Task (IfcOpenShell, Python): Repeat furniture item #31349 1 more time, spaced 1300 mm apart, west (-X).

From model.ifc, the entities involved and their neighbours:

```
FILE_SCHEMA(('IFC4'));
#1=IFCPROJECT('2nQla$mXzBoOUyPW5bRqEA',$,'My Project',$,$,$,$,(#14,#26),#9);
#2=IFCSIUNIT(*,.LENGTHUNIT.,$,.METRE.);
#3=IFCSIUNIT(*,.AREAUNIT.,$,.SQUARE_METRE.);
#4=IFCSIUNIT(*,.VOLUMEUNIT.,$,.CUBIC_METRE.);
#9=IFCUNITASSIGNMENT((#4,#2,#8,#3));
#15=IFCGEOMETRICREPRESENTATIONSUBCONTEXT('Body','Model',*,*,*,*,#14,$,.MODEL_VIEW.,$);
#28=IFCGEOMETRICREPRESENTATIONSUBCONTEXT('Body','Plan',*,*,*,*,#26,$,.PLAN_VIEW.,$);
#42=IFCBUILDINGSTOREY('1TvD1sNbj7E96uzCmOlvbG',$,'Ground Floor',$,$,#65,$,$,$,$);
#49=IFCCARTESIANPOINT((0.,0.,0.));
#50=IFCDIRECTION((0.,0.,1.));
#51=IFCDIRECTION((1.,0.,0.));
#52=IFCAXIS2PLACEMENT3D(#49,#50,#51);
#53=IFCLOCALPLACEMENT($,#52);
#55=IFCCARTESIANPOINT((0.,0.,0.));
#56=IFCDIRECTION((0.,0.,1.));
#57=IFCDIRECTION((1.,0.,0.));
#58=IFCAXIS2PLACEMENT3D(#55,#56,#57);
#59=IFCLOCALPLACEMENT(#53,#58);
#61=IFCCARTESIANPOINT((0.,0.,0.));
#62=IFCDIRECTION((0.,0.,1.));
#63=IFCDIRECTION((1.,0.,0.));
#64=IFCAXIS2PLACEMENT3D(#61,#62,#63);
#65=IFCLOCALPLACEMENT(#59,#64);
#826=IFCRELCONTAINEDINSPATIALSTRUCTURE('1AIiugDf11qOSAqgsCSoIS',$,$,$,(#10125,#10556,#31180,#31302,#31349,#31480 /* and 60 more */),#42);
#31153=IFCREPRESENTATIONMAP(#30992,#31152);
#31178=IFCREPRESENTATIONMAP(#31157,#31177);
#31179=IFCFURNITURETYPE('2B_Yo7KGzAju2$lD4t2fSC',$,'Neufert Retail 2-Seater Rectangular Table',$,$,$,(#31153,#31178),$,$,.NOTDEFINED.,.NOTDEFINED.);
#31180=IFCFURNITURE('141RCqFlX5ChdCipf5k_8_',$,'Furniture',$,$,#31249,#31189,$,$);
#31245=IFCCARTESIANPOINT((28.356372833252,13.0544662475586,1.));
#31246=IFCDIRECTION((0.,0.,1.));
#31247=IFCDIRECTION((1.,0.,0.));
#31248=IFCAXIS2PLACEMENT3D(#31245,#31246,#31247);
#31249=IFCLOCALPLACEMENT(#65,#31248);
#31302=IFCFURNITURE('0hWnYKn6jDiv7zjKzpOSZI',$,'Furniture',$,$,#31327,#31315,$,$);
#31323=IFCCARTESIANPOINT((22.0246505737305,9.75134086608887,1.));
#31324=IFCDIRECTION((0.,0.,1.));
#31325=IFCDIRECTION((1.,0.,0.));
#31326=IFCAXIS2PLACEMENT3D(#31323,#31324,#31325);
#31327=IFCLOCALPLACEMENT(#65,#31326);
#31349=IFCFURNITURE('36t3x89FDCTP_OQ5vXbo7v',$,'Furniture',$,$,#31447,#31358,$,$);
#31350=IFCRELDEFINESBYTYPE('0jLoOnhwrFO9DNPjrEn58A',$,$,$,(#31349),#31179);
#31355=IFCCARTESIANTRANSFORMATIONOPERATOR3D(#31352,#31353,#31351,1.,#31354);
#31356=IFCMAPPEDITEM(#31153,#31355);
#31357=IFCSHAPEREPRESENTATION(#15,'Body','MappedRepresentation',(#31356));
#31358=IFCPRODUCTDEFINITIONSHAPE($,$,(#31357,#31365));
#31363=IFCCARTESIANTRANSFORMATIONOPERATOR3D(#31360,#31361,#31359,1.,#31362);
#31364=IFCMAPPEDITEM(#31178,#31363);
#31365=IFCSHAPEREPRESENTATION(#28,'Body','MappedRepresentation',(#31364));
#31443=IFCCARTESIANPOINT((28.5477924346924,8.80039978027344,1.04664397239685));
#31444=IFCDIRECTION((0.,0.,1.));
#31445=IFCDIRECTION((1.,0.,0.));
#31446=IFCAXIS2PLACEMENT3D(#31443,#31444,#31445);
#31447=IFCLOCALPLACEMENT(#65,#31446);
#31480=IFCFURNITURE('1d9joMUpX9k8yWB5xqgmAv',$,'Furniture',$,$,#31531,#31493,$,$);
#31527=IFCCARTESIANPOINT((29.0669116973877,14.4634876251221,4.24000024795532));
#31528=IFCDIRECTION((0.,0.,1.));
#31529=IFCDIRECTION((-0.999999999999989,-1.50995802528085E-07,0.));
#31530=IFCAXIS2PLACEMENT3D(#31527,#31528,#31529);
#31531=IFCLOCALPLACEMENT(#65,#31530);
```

```python
import numpy as np
import ifcopenshell
import ifcopenshell.api.geometry
import ifcopenshell.api.root
import ifcopenshell.util.element
import ifcopenshell.util.placement
import ifcopenshell.util.unit

model = ifcopenshell.open("model.ifc")
unit_scale = ifcopenshell.util.unit.calculate_unit_scale(model)

source = model.by_guid("36t3x89FDCTP_OQ5vXbo7v")
base = ifcopenshell.util.placement.get_local_placement(source.ObjectPlacement)
step = np.array([-1.0, 0.0, 0.0]) * 1.3 / unit_scale

for i in range(1, 2):
    copy = ifcopenshell.api.root.copy_class(model, product=source)
    copy.Representation = ifcopenshell.util.element.copy_deep(
        model, source.Representation, exclude=["IfcGeometricRepresentationContext", "IfcRepresentationMap"]
    )
    matrix = base.copy()
    matrix[:3, 3] += i * step
    print("added at", matrix[:3, 3].round(3) + 0.0)
    ifcopenshell.api.geometry.edit_object_placement(model, product=copy, matrix=matrix, is_si=False)

model.write("model_v2.ifc")
```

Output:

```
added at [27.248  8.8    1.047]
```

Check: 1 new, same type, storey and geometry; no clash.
